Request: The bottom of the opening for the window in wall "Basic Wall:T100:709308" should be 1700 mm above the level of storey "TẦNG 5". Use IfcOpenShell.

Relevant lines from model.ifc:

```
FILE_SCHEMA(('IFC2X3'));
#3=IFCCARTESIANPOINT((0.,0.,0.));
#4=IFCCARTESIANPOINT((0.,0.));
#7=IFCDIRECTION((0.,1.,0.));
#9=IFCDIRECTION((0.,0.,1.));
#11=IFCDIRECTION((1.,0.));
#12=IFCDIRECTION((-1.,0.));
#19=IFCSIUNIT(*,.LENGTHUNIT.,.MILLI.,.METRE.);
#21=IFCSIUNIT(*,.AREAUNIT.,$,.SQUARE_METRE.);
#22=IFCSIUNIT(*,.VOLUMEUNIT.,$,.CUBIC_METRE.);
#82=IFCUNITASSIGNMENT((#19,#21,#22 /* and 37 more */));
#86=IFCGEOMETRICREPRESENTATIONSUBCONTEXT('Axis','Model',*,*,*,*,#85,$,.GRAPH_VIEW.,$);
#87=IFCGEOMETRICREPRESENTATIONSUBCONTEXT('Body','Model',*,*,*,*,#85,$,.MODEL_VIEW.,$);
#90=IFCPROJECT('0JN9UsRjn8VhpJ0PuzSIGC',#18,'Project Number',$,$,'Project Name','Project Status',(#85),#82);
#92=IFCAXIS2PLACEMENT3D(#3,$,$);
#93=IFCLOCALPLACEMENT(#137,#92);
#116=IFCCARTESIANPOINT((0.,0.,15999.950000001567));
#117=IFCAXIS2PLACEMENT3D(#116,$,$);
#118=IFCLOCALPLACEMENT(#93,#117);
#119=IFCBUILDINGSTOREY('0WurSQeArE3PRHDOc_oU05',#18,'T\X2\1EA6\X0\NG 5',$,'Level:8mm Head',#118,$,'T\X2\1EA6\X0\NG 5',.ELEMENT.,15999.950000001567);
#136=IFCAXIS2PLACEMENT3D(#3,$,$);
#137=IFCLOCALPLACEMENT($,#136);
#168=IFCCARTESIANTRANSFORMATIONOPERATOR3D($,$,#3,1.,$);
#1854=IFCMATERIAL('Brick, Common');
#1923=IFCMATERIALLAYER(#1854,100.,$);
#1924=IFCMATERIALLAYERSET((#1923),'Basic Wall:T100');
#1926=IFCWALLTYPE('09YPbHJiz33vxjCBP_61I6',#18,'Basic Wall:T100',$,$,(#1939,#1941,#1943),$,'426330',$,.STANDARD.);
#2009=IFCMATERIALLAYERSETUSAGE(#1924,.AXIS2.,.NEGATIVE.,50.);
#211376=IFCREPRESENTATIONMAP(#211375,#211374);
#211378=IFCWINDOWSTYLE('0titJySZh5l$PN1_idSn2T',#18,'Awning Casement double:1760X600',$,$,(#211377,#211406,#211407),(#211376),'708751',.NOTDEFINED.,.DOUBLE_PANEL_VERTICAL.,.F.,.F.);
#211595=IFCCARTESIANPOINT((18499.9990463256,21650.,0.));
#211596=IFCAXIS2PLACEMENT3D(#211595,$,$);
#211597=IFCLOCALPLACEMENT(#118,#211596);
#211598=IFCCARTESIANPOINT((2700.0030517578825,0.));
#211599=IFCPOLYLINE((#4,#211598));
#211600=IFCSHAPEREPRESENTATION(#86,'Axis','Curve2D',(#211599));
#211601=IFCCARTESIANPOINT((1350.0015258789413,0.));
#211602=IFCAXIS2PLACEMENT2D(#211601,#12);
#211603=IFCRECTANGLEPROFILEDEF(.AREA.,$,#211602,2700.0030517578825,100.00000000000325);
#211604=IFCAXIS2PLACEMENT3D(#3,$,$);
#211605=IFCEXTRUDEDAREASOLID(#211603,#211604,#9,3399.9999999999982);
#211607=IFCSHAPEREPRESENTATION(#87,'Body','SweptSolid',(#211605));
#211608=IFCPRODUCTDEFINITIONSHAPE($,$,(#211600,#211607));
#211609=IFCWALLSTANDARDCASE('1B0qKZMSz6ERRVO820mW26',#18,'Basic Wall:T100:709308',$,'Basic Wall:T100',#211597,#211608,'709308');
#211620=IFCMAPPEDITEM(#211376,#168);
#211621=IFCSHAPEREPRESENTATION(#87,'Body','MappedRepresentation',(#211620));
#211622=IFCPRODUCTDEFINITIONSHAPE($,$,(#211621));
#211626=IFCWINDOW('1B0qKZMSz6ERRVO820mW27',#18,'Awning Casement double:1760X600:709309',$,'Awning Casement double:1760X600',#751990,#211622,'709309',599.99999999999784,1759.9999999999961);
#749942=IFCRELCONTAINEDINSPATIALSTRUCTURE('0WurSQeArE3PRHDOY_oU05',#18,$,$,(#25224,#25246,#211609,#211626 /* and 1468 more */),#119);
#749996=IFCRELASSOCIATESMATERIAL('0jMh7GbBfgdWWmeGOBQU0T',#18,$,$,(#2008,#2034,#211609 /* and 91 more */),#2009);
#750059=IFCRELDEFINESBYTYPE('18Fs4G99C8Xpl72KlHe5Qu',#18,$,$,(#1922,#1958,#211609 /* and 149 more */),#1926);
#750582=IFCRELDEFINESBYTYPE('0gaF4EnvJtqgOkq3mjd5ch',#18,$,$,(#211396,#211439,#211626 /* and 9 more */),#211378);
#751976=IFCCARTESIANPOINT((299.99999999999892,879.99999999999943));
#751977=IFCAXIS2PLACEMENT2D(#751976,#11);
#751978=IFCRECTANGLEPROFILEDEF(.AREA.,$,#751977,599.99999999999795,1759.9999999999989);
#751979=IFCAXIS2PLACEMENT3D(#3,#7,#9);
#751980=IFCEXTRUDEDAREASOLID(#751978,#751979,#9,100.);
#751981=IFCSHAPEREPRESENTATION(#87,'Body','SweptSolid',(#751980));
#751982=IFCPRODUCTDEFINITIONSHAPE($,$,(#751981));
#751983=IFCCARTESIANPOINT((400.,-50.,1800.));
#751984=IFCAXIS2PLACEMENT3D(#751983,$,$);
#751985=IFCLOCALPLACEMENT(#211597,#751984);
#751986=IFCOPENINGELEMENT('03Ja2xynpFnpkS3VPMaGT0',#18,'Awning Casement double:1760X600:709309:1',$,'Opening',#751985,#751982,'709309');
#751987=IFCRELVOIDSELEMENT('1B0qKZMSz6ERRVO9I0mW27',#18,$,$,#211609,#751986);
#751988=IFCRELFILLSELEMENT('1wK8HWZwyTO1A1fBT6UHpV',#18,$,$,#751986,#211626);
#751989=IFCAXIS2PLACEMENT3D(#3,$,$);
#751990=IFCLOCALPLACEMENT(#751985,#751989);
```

```python
import numpy as np
import ifcopenshell
import ifcopenshell.api.geometry
import ifcopenshell.geom
import ifcopenshell.util.element
import ifcopenshell.util.placement
import ifcopenshell.util.shape
import ifcopenshell.util.unit

model = ifcopenshell.open("model.ifc")
unit_scale = ifcopenshell.util.unit.calculate_unit_scale(model)

window = model.by_guid("1B0qKZMSz6ERRVO820mW27")
opening = window.FillsVoids[0].RelatingOpeningElement
storey = ifcopenshell.util.element.get_container(window, ifc_class="IfcBuildingStorey")
level = ifcopenshell.util.placement.get_local_placement(storey.ObjectPlacement)[2, 3]

# The opening's origin need not be at the sill, so measure its lowest point.
shape = ifcopenshell.geom.create_shape(ifcopenshell.geom.settings(), opening)
bottom = ifcopenshell.util.shape.get_shape_bottom_elevation(shape, shape.geometry) / unit_scale
dz = level + 1700.0 - bottom

shift = np.array([0.0, 0.0, dz])
# The window is placed relative to its opening, so it follows when the opening moves.
matrix = ifcopenshell.util.placement.get_local_placement(opening.ObjectPlacement)
matrix[:3, 3] += shift
ifcopenshell.api.geometry.edit_object_placement(
    model, product=opening, matrix=matrix, is_si=False, should_transform_children=True
)

print(f"moved by {dz * unit_scale:+.3f} m")

model.write("model-out.ifc")
```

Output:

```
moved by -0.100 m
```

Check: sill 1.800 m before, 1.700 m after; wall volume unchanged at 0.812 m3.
